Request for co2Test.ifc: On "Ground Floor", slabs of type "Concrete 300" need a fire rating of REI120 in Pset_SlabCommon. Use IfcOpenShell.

First a look at what the model holds.

```python
import ifcopenshell
import ifcopenshell.util.element

model = ifcopenshell.open("co2Test.ifc")
print(model.schema)
storey = next(s for s in model.by_type("IfcBuildingStorey") if s.Name == "Ground Floor")
slabs = [e for e in ifcopenshell.util.element.get_decomposition(storey) if e.is_a("IfcSlab")]
seen = {}
for e in slabs:
    element_type = ifcopenshell.util.element.get_type(e)
    key = (element_type.Name if element_type != e and element_type else None, ifcopenshell.util.element.get_pset(e, "Pset_SlabCommon", "FireRating"))
    seen[key] = seen.get(key, 0) + 1
for (name, value), count in sorted(seen.items(), key=str):
    print(count, "x", name, "|", value)
```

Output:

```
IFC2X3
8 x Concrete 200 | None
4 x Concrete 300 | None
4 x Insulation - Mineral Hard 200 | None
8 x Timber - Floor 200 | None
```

```python
import ifcopenshell
import ifcopenshell.api.pset
import ifcopenshell.util.element

model = ifcopenshell.open("co2Test.ifc")

storey = next(s for s in model.by_type("IfcBuildingStorey") if s.Name == "Ground Floor")
slabs = [e for e in ifcopenshell.util.element.get_decomposition(storey) if e.is_a("IfcSlab")]

count = 0
for e in slabs:
    element_type = ifcopenshell.util.element.get_type(e)
    if element_type in (None, e) or element_type.Name != "Concrete 300":
        continue
    # add_pset returns the element's existing set when there is one.
    pset = ifcopenshell.api.pset.add_pset(model, product=e, name="Pset_SlabCommon")
    ifcopenshell.api.pset.edit_pset(model, pset=pset, properties={"FireRating": "REI120"})
    count += 1

print(count, "slabs updated")

model.write("co2Test_edited.ifc")
```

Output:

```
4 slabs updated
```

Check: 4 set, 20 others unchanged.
